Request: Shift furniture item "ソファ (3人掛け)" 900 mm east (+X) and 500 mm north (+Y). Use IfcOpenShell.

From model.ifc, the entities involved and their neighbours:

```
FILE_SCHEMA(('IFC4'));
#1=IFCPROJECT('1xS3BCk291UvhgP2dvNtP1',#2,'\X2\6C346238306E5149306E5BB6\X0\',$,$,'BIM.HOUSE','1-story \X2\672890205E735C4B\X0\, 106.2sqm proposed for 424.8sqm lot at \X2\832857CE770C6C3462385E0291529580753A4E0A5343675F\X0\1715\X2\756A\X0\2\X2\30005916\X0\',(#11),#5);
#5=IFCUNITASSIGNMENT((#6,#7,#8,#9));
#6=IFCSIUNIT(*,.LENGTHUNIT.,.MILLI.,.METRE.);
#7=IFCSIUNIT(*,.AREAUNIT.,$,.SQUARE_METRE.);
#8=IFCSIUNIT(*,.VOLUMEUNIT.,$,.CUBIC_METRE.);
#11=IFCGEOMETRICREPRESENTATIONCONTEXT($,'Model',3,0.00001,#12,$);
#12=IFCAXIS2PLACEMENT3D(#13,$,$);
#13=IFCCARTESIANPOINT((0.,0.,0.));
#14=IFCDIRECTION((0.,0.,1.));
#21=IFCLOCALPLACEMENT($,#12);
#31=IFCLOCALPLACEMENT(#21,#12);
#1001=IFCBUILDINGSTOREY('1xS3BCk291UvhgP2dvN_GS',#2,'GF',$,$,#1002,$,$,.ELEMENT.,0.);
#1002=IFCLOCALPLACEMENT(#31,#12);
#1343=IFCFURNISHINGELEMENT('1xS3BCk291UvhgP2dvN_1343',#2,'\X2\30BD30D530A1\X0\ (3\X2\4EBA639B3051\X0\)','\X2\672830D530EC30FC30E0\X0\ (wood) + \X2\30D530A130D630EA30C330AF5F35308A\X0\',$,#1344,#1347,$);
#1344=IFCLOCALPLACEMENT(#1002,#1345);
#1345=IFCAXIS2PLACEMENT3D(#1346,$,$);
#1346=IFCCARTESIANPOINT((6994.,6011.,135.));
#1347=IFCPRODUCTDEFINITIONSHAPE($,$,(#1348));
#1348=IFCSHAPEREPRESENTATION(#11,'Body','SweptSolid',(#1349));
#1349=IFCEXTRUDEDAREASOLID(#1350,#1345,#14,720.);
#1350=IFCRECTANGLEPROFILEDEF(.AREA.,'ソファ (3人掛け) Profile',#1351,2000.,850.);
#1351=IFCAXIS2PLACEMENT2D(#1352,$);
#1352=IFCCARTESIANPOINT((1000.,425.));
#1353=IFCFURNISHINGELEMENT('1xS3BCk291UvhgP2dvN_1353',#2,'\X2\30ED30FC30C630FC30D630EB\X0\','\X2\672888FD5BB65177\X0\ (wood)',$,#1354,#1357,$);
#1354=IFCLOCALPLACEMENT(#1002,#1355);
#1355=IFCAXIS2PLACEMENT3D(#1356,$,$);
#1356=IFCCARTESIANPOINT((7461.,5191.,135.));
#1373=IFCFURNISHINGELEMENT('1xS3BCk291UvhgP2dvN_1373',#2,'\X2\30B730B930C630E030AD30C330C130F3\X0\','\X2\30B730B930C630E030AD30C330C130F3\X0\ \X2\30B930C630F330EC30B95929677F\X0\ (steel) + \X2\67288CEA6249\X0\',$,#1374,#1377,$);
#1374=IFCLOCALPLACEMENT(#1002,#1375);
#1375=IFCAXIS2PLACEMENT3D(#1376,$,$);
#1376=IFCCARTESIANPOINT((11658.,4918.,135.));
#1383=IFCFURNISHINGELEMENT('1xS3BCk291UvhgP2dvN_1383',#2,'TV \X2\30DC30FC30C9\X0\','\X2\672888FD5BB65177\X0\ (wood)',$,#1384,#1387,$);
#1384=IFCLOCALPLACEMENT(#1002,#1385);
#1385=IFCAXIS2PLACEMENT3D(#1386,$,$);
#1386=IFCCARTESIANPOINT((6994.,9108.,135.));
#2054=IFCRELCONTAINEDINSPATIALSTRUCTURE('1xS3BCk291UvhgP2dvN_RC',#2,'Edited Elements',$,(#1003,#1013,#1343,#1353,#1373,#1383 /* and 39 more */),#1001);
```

```python
import ifcopenshell
import ifcopenshell.api.geometry
import ifcopenshell.util.placement

model = ifcopenshell.open("model.ifc")

item = model.by_guid("1xS3BCk291UvhgP2dvN_1343")
matrix = ifcopenshell.util.placement.get_local_placement(item.ObjectPlacement)
matrix[0, 3] += 900.0
matrix[1, 3] += 500.0
ifcopenshell.api.geometry.edit_object_placement(model, product=item, matrix=matrix, is_si=False)

print(ifcopenshell.util.placement.get_local_placement(item.ObjectPlacement).round(3) + 0.0)

model.write("model_rev.ifc")
```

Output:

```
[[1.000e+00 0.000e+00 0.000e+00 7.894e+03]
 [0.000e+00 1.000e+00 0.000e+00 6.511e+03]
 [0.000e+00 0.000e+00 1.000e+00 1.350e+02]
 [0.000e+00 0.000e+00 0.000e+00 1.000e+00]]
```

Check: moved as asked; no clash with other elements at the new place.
